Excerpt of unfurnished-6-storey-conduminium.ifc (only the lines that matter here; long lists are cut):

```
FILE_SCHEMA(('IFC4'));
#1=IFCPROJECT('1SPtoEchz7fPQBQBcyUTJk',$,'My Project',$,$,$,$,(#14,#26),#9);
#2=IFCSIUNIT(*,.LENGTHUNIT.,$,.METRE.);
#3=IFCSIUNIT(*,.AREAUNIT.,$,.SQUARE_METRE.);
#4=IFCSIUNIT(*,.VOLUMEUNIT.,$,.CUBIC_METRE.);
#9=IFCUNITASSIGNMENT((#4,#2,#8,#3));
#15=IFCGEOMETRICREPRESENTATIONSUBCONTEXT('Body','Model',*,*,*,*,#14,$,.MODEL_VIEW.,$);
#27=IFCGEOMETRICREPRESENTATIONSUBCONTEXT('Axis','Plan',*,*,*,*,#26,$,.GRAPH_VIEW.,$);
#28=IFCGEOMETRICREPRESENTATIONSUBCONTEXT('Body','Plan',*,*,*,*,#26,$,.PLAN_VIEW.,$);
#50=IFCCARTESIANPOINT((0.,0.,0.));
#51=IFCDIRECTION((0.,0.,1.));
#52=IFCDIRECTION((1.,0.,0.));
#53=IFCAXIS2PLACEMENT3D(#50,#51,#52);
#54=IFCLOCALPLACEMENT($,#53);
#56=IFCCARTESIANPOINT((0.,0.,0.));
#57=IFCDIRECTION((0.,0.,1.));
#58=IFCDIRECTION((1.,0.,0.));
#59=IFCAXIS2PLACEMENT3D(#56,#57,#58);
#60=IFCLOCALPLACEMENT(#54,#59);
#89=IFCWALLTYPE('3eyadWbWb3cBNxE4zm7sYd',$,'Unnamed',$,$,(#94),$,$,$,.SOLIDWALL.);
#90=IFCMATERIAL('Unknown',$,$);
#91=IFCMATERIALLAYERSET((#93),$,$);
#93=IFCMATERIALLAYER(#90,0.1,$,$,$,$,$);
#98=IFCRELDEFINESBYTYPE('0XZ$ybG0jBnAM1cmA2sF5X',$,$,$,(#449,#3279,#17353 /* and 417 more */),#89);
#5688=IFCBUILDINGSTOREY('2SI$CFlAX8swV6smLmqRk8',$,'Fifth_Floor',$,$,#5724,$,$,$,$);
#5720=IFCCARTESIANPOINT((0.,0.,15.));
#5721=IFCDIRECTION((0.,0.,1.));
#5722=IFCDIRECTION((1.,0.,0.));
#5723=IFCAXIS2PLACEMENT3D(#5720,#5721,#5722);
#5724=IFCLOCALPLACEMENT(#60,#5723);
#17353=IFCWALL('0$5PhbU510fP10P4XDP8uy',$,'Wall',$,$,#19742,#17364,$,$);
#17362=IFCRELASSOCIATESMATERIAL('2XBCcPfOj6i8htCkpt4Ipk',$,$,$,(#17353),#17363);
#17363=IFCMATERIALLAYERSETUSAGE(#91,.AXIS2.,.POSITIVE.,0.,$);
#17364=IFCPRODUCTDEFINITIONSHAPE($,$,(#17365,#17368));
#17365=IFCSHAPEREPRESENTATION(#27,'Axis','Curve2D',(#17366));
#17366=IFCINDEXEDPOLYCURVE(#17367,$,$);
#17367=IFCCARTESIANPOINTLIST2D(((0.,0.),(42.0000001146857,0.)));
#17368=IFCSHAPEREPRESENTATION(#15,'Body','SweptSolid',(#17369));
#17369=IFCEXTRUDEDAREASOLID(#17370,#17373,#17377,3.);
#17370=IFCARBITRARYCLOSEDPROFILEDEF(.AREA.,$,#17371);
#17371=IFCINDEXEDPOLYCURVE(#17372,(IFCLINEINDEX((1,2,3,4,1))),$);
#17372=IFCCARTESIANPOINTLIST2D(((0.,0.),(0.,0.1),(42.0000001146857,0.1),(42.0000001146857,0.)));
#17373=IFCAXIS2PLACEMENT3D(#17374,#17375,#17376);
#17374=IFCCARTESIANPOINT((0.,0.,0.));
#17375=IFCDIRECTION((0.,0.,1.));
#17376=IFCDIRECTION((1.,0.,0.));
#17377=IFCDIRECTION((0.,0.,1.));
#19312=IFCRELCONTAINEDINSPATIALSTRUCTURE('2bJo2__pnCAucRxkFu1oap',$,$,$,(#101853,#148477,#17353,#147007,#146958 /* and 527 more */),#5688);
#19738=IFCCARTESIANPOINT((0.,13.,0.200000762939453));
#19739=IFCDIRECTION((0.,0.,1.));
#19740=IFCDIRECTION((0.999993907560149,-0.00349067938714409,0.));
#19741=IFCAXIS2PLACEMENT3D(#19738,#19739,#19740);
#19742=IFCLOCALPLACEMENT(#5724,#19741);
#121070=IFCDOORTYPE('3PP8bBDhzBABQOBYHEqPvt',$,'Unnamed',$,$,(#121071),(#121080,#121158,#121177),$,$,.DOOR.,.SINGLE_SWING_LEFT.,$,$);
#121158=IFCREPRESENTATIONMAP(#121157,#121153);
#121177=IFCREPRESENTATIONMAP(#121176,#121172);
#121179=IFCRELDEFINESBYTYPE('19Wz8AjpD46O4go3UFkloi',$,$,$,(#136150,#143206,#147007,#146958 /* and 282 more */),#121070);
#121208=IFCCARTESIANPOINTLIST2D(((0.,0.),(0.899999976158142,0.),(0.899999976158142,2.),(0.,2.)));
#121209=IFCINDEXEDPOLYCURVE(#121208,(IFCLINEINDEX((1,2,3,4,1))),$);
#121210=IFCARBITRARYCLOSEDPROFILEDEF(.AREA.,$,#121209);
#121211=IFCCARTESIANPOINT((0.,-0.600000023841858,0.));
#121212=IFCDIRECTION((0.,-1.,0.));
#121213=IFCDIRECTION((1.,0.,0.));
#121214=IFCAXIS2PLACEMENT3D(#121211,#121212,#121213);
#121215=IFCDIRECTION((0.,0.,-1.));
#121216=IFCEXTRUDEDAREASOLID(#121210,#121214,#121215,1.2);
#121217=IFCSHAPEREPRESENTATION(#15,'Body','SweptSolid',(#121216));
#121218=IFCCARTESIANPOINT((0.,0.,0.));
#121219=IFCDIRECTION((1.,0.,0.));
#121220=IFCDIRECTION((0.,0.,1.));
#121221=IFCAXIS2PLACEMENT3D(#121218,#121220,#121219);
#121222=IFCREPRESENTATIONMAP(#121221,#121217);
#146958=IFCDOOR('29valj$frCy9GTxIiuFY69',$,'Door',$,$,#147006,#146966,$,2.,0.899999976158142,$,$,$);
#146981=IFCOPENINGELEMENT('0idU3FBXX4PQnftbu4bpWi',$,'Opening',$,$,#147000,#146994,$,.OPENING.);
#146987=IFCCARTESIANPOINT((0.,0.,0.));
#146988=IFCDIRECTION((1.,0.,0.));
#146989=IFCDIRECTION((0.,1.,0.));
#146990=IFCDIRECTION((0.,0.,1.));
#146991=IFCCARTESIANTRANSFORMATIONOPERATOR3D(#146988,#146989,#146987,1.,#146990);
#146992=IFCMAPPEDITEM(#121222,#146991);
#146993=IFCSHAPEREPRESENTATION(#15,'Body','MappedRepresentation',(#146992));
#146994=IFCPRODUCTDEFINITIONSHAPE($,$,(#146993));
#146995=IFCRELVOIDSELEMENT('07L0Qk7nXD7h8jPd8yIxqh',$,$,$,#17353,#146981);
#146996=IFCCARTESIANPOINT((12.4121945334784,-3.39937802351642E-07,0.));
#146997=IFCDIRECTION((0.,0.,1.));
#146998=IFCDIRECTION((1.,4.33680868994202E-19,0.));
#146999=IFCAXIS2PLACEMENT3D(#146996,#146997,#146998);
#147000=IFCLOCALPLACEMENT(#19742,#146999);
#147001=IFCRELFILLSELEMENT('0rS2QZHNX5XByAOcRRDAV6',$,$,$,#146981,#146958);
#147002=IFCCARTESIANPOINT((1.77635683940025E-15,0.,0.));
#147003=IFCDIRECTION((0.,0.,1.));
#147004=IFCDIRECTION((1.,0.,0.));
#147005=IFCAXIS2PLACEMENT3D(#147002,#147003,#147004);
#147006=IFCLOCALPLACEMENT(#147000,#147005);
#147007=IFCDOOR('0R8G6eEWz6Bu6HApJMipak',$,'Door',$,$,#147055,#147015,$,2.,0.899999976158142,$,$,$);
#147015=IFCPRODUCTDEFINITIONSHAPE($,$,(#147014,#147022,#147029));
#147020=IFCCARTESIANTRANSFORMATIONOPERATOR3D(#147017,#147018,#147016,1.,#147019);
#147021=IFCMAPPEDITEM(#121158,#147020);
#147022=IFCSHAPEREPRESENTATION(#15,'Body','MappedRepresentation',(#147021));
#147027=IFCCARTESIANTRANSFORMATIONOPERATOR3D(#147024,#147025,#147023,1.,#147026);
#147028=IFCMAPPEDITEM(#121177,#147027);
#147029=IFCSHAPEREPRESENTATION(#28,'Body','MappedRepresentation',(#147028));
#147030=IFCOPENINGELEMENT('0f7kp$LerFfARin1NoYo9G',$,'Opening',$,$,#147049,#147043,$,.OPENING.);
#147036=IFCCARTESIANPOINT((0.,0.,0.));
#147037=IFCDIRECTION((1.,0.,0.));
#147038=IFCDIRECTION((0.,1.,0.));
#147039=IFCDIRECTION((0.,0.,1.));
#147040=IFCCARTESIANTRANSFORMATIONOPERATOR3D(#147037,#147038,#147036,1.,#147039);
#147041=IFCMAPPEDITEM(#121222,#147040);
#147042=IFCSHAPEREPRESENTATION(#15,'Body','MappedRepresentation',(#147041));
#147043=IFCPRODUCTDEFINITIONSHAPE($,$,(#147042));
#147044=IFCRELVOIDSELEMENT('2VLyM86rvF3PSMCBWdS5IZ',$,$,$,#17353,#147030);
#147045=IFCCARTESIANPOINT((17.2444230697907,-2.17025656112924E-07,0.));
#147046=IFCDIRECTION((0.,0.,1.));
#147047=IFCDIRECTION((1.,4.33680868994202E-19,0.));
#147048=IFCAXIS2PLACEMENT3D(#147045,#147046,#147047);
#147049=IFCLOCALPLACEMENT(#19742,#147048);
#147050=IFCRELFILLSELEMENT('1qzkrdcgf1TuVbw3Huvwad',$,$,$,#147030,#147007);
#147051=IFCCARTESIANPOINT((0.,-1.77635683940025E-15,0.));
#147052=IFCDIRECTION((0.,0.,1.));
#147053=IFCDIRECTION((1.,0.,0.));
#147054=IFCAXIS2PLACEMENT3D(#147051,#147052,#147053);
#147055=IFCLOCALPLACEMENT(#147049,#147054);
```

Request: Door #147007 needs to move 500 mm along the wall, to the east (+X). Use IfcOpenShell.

```python
import ifcopenshell
import ifcopenshell.api.geometry
import ifcopenshell.util.placement

model = ifcopenshell.open("unfurnished-6-storey-conduminium.ifc")

door = model.by_guid("0R8G6eEWz6Bu6HApJMipak")
opening = door.FillsVoids[0].RelatingOpeningElement
wall = opening.VoidsElements[0].RelatingBuildingElement

wall_matrix = ifcopenshell.util.placement.get_local_placement(wall.ObjectPlacement)
shift = wall_matrix[:3, 0] * 0.5
before = ifcopenshell.util.placement.get_local_placement(door.ObjectPlacement)[:3, 3].copy()

# The door is placed relative to its opening, so it follows when the opening moves.
matrix = ifcopenshell.util.placement.get_local_placement(opening.ObjectPlacement)
matrix[:3, 3] += shift
ifcopenshell.api.geometry.edit_object_placement(
    model, product=opening, matrix=matrix, is_si=False, should_transform_children=True
)

after = ifcopenshell.util.placement.get_local_placement(door.ObjectPlacement)[:3, 3]
print("door moved by", (after - before).round(3) + 0.0)

model.write("unfurnished-6-storey-conduminium_v2.ifc")
```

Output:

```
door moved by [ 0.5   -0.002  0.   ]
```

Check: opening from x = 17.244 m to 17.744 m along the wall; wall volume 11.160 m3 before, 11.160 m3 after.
